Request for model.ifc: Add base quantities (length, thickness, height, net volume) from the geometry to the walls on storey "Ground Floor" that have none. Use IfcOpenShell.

First a look at what the model holds.

```python
import ifcopenshell
import ifcopenshell.util.element
import ifcopenshell.util.unit

model = ifcopenshell.open("model.ifc")
print(model.schema)
for unit_type in ("LENGTHUNIT", "AREAUNIT", "VOLUMEUNIT"):
    print(unit_type, ifcopenshell.util.unit.calculate_unit_scale(model, unit_type))
storey = next(s for s in model.by_type("IfcBuildingStorey") if s.Name == "Ground Floor")
walls = [e for e in ifcopenshell.util.element.get_decomposition(storey) if e.is_a("IfcWall")]
for e in sorted(walls, key=lambda e: e.id()):
    print(e.id(), e.is_a(), e.Name, list(ifcopenshell.util.element.get_psets(e, qtos_only=True)), sep=" | ")
```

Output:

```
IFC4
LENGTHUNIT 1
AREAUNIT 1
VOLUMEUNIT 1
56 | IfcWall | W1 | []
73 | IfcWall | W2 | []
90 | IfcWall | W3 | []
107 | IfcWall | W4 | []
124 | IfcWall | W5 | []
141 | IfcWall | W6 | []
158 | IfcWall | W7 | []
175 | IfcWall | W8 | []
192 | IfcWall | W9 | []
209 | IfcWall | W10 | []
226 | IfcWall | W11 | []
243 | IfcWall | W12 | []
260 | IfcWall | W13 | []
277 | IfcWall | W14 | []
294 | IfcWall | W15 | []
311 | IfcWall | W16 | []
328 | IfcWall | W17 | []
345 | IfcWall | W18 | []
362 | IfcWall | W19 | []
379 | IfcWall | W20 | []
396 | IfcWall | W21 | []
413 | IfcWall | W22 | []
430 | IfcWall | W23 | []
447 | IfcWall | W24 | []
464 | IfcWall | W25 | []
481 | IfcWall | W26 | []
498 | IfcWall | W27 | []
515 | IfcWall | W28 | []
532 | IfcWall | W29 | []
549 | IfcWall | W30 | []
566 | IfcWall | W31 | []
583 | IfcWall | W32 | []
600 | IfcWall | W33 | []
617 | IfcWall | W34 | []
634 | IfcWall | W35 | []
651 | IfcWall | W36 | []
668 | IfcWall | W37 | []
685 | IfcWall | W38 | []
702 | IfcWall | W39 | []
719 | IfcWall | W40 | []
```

```python
import ifcopenshell
import ifcopenshell.api.pset
import ifcopenshell.geom
import ifcopenshell.util.element
import ifcopenshell.util.shape
import ifcopenshell.util.unit

model = ifcopenshell.open("model.ifc")
unit_scale = ifcopenshell.util.unit.calculate_unit_scale(model)
volume_scale = ifcopenshell.util.unit.calculate_unit_scale(model, "VOLUMEUNIT")
settings = ifcopenshell.geom.settings()

storey = next(s for s in model.by_type("IfcBuildingStorey") if s.Name == "Ground Floor")
walls = [e for e in ifcopenshell.util.element.get_decomposition(storey) if e.is_a("IfcWall")]

for e in sorted(walls, key=lambda e: e.id()):
    if ifcopenshell.util.element.get_psets(e, qtos_only=True, should_inherit=False):
        continue
    # Geometry comes back in metres, in the element's own axes.
    shape = ifcopenshell.geom.create_shape(settings, e)
    values = {
        "Length": ifcopenshell.util.shape.get_x(shape.geometry) / unit_scale,
        "Width": ifcopenshell.util.shape.get_y(shape.geometry) / unit_scale,
        "Height": ifcopenshell.util.shape.get_z(shape.geometry) / unit_scale,
        "NetVolume": ifcopenshell.util.shape.get_volume(shape.geometry) / volume_scale,
    }
    qto = ifcopenshell.api.pset.add_qto(model, product=e, name="Qto_WallBaseQuantities")
    ifcopenshell.api.pset.edit_qto(model, qto=qto, properties=values)
    print(e.id(), {k: round(v, 3) for k, v in values.items()})

model.write("model_updated.ifc")
```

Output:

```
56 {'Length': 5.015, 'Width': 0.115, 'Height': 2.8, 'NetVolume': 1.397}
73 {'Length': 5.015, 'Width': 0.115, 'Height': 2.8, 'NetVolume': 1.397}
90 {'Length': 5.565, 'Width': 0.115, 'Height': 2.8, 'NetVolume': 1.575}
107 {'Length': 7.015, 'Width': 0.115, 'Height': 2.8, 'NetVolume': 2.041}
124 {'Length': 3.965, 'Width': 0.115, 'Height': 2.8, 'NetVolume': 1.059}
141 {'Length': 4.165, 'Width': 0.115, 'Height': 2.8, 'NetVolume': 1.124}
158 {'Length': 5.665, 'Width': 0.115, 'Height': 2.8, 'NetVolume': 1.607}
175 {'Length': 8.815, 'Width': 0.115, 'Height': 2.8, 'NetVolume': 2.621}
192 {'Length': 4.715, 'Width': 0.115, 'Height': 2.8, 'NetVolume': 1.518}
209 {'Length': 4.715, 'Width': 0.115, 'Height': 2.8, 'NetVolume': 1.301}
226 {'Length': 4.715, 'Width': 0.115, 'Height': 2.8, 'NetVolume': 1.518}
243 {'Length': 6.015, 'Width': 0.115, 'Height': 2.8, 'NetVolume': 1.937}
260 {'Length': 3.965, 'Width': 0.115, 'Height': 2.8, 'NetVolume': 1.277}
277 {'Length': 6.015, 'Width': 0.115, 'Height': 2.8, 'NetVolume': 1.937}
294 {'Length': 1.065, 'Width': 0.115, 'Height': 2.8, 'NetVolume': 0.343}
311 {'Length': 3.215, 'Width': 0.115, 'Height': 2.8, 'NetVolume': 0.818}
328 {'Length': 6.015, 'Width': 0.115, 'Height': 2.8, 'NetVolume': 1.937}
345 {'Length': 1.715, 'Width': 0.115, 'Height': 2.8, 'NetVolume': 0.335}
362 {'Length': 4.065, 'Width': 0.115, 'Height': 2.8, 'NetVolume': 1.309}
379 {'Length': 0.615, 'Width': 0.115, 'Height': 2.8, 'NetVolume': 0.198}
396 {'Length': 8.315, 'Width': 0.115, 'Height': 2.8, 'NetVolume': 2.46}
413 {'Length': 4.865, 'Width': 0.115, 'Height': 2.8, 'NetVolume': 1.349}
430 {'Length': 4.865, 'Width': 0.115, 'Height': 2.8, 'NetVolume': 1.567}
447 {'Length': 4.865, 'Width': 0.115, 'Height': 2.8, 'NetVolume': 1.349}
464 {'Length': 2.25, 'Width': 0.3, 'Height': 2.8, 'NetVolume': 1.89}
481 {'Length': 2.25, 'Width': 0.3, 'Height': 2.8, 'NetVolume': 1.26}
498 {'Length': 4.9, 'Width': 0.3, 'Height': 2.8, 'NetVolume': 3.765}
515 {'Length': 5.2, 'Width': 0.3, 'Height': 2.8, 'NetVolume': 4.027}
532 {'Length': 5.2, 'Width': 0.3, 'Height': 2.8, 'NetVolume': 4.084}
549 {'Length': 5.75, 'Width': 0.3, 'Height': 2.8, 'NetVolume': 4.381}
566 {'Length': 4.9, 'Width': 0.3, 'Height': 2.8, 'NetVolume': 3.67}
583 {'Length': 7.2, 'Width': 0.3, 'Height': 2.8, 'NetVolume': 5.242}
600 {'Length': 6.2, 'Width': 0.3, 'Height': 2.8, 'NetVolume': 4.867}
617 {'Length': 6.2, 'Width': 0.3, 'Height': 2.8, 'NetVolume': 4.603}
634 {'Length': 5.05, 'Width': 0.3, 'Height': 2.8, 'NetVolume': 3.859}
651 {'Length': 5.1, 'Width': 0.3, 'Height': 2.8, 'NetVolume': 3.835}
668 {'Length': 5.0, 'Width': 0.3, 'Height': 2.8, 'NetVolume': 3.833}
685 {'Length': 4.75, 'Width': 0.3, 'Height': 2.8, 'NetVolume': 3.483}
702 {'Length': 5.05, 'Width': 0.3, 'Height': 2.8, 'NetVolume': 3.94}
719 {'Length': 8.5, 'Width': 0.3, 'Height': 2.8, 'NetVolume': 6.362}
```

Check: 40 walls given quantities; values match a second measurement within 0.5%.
